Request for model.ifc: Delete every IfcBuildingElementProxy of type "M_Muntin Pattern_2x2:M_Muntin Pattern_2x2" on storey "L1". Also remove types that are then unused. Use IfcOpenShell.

First a look at what the model holds.

```python
import ifcopenshell
import ifcopenshell.util.element

model = ifcopenshell.open("model.ifc")
print(model.schema)
storey = next(s for s in model.by_type("IfcBuildingStorey") if s.Name == "L1")
proxies = [e for e in ifcopenshell.util.element.get_decomposition(storey) if e.is_a("IfcBuildingElementProxy")]
seen = {}
for e in proxies:
    element_type = ifcopenshell.util.element.get_type(e)
    name = element_type.Name if element_type not in (None, e) else None
    seen[name] = seen.get(name, 0) + 1
for name, count in sorted(seen.items(), key=str):
    print(count, "x", name)
```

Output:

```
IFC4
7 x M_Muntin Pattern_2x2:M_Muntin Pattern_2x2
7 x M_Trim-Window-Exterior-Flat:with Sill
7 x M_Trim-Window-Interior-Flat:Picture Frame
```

```python
import ifcopenshell
import ifcopenshell.api.root
import ifcopenshell.util.element

model = ifcopenshell.open("model.ifc")

storey = next(s for s in model.by_type("IfcBuildingStorey") if s.Name == "L1")
proxies = [e for e in ifcopenshell.util.element.get_decomposition(storey) if e.is_a("IfcBuildingElementProxy")]
targets = [e for e in proxies if (t := ifcopenshell.util.element.get_type(e)) not in (None, e) and t.Name == "M_Muntin Pattern_2x2:M_Muntin Pattern_2x2"]
types = {ifcopenshell.util.element.get_type(e) for e in targets} - {None, *targets}

for e in targets:
    ifcopenshell.api.root.remove_product(model, product=e)
print(len(targets), "removed")

unused = [t for t in types if not ifcopenshell.util.element.get_types(t)]
for t in unused:
    ifcopenshell.api.root.remove_product(model, product=t)
print(len(unused), "unused types removed")

model.write("model_updated.ifc")
```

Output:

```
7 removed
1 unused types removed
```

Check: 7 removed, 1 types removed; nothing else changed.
